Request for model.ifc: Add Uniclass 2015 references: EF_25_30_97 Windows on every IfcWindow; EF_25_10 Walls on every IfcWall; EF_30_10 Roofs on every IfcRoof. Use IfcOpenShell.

First a look at what the model holds.

```python
import ifcopenshell

model = ifcopenshell.open("model.ifc")
print(model.schema)
print("classifications:", [c.Name for c in model.by_type("IfcClassification")])
for ifc_class in ("IfcDoor", "IfcRoof", "IfcStair", "IfcWall", "IfcWindow"):
    print(ifc_class, len(model.by_type(ifc_class)))
```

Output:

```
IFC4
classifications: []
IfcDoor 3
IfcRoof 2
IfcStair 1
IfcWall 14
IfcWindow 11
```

```python
import ifcopenshell
import ifcopenshell.api.classification

model = ifcopenshell.open("model.ifc")

system = ifcopenshell.api.classification.add_classification(model, classification="Uniclass 2015")

codes = {
    "IfcWindow": ("EF_25_30_97", "Windows"),
    "IfcWall": ("EF_25_10", "Walls"),
    "IfcRoof": ("EF_30_10", "Roofs"),
}
for ifc_class, (code, name) in codes.items():
    products = model.by_type(ifc_class)
    ifcopenshell.api.classification.add_reference(
        model, products=products, classification=system, identification=code, name=name
    )
    print(code, len(products))

model.write("model_v2.ifc")
```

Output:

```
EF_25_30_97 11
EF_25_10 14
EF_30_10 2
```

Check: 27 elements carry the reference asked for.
